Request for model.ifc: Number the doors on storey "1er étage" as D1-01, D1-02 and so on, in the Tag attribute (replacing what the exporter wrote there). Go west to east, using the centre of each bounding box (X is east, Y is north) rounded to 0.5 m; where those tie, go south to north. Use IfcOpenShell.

First a look at what the model holds.

```python
import ifcopenshell
import ifcopenshell.util.element
import ifcopenshell.util.placement

model = ifcopenshell.open("model.ifc")
print(model.schema)
storey = next(s for s in model.by_type("IfcBuildingStorey") if s.Name == "1er étage")
doors = [e for e in ifcopenshell.util.element.get_decomposition(storey) if e.is_a("IfcDoor")]
for e in sorted(doors, key=lambda e: e.id()):
    origin = ifcopenshell.util.placement.get_local_placement(e.ObjectPlacement)[:3, 3]
    print(e.id(), e.Tag, e.Name, origin.round(2) + 0.0, sep=" | ")
```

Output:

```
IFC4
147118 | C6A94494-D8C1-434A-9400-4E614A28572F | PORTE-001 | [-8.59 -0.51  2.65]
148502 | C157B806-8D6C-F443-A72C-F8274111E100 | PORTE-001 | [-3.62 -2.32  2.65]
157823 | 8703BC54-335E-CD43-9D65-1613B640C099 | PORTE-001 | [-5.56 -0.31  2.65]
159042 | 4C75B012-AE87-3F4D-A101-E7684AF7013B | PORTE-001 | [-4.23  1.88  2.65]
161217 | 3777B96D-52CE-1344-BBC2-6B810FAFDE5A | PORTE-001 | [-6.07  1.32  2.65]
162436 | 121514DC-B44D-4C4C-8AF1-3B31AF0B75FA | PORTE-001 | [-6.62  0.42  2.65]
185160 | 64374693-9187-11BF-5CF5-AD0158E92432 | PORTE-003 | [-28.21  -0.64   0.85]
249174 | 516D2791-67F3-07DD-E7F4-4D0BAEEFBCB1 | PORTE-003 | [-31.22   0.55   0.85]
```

```python
import ifcopenshell
import ifcopenshell.geom
import ifcopenshell.util.element
import ifcopenshell.util.shape

model = ifcopenshell.open("model.ifc")
settings = ifcopenshell.geom.settings()
settings.set("use-world-coords", True)


def centre(element):
    shape = ifcopenshell.geom.create_shape(settings, element)
    return ifcopenshell.util.shape.get_bbox_centroid(shape.geometry)


storey = next(s for s in model.by_type("IfcBuildingStorey") if s.Name == "1er étage")
doors = [e for e in ifcopenshell.util.element.get_decomposition(storey) if e.is_a("IfcDoor")]

# Insertion points can sit at a corner or the storey origin, so sort by the geometry (in metres).
centres = {e: centre(e) for e in doors}
doors.sort(key=lambda e: (round(centres[e][0] / 0.5), centres[e][1]))

for i, e in enumerate(doors, start=1):
    number = f"D1-{i:02d}"
    e.Tag = number
    print(e.id(), number)

model.write("model_updated.ifc")
```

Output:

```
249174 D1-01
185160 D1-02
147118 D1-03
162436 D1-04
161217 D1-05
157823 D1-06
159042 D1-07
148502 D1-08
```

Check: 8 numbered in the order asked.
